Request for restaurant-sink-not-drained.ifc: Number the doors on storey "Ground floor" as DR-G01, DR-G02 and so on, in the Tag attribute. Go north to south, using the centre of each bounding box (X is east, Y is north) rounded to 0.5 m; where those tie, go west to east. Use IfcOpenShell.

First a look at what the model holds.

```python
import ifcopenshell
import ifcopenshell.util.element
import ifcopenshell.util.placement

model = ifcopenshell.open("restaurant-sink-not-drained.ifc")
print(model.schema)
storey = next(s for s in model.by_type("IfcBuildingStorey") if s.Name == "Ground floor")
doors = [e for e in ifcopenshell.util.element.get_decomposition(storey) if e.is_a("IfcDoor")]
for e in sorted(doors, key=lambda e: e.id()):
    origin = ifcopenshell.util.placement.get_local_placement(e.ObjectPlacement)[:3, 3]
    print(e.id(), e.Tag, e.Name, origin.round(2) + 0.0, sep=" | ")
```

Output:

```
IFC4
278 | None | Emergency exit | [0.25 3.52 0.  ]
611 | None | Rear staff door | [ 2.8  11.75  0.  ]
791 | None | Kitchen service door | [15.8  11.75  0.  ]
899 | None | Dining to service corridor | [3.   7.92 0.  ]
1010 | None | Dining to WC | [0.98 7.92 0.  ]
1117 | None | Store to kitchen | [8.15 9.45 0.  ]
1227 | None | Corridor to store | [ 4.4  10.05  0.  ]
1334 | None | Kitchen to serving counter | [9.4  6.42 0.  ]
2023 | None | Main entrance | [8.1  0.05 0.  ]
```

```python
import ifcopenshell
import ifcopenshell.geom
import ifcopenshell.util.element
import ifcopenshell.util.shape

model = ifcopenshell.open("restaurant-sink-not-drained.ifc")
settings = ifcopenshell.geom.settings()
settings.set("use-world-coords", True)


def centre(element):
    shape = ifcopenshell.geom.create_shape(settings, element)
    return ifcopenshell.util.shape.get_bbox_centroid(shape.geometry)


storey = next(s for s in model.by_type("IfcBuildingStorey") if s.Name == "Ground floor")
doors = [e for e in ifcopenshell.util.element.get_decomposition(storey) if e.is_a("IfcDoor")]

# Insertion points can sit at a corner or the storey origin, so sort by the geometry (in metres).
centres = {e: centre(e) for e in doors}
doors.sort(key=lambda e: (-round(centres[e][1] / 0.5), centres[e][0]))

for i, e in enumerate(doors, start=1):
    number = f"DR-G{i:02d}"
    e.Tag = number
    print(e.id(), number)

model.write("restaurant-sink-not-drained_v2.ifc")
```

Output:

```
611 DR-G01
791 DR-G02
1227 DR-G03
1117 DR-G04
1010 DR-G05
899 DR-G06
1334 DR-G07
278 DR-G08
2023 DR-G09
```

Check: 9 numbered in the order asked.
